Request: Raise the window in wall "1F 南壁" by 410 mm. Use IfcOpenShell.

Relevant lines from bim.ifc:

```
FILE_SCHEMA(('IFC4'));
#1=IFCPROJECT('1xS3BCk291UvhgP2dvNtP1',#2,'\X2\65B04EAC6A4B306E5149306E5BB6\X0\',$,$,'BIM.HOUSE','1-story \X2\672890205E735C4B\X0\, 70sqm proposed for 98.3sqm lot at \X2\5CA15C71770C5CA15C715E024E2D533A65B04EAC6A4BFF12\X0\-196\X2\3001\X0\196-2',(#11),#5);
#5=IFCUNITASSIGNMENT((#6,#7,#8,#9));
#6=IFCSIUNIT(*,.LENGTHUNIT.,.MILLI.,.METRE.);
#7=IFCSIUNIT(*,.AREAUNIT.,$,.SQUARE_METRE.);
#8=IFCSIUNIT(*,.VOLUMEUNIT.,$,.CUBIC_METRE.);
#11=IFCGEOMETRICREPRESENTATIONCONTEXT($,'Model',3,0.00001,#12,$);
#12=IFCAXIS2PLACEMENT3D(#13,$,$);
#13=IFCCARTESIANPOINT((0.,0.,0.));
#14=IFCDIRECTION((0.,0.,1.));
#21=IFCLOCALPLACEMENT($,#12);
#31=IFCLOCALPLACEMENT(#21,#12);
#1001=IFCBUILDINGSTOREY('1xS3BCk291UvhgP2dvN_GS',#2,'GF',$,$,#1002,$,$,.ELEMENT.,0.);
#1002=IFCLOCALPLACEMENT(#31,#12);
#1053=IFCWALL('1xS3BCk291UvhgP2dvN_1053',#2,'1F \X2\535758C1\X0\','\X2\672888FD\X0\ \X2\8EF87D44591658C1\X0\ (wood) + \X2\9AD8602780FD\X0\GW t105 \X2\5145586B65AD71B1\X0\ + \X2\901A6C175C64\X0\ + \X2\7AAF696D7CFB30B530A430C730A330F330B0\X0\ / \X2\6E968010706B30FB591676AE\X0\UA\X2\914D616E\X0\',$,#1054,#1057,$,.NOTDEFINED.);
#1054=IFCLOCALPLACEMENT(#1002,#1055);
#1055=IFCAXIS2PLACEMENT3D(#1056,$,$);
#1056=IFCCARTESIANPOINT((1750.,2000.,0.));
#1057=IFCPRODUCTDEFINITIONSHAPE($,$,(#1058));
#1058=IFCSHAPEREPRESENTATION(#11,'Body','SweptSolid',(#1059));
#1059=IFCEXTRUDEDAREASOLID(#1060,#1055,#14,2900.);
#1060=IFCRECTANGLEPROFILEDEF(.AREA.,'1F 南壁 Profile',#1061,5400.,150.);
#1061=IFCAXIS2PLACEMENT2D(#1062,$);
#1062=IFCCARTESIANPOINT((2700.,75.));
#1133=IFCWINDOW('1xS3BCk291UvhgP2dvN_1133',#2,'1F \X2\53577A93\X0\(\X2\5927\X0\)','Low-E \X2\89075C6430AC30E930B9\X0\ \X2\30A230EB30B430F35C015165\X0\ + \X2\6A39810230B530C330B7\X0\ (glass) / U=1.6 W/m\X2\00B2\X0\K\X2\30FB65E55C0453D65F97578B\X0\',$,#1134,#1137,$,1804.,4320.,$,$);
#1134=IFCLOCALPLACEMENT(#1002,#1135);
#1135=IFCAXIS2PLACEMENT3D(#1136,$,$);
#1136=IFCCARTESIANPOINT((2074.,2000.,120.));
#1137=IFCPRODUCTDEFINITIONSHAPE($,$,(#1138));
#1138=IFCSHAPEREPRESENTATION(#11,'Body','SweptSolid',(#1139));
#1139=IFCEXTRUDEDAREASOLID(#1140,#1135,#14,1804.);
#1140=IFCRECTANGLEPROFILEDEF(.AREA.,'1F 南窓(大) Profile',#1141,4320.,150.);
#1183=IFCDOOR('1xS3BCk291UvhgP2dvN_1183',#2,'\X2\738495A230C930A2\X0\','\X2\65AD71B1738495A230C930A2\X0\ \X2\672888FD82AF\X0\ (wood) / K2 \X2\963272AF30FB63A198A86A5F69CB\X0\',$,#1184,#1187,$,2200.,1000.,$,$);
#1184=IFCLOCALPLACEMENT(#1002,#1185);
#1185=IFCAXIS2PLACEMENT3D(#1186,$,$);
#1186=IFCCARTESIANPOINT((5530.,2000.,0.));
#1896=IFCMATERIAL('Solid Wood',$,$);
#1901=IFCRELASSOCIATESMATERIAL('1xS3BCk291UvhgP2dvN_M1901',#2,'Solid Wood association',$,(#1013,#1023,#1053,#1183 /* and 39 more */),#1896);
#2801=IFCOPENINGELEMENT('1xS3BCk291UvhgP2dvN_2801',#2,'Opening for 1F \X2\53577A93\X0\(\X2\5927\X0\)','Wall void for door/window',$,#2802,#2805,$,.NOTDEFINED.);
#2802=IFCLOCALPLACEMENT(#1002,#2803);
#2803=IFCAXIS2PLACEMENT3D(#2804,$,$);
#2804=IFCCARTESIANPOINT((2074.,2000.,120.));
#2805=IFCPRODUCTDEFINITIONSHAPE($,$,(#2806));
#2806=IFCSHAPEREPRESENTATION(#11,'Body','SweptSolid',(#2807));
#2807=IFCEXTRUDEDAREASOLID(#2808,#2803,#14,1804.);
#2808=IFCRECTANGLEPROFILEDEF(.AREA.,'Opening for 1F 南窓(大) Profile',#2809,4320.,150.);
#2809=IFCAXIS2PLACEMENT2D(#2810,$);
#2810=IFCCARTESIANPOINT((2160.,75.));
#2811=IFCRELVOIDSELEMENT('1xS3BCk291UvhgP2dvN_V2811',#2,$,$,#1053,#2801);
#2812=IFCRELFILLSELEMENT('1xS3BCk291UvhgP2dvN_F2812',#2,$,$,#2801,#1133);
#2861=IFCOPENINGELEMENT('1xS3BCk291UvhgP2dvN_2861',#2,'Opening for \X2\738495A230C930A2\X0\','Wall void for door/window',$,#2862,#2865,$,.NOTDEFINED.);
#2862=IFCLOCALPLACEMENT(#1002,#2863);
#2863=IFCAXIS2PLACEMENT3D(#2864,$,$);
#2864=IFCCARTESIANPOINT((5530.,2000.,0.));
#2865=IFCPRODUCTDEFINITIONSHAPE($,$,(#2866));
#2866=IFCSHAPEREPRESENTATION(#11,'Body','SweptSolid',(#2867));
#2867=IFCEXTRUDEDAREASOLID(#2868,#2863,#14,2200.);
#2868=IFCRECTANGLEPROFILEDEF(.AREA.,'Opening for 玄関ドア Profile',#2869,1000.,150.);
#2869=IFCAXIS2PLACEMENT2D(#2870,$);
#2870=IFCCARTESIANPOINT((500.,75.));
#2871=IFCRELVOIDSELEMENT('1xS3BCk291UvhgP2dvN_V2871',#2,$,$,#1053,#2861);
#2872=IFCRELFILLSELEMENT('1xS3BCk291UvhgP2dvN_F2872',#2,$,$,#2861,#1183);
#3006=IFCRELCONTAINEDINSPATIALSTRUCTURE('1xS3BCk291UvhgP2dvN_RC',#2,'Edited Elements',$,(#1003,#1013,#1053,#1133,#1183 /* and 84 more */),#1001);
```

```python
import numpy as np
import ifcopenshell
import ifcopenshell.api.geometry
import ifcopenshell.util.placement
import ifcopenshell.util.unit

model = ifcopenshell.open("bim.ifc")
unit_scale = ifcopenshell.util.unit.calculate_unit_scale(model)

window = model.by_id(1133)
opening = window.FillsVoids[0].RelatingOpeningElement
dz = 0.41 / unit_scale

shift = np.array([0.0, 0.0, dz])
# The window is not placed relative to its opening, so move both.
for product in (opening, window):
    matrix = ifcopenshell.util.placement.get_local_placement(product.ObjectPlacement)
    matrix[:3, 3] += shift
    ifcopenshell.api.geometry.edit_object_placement(model, product=product, matrix=matrix, is_si=False)

print(f"moved by {dz * unit_scale:+.3f} m")

model.write("bim_updated.ifc")
```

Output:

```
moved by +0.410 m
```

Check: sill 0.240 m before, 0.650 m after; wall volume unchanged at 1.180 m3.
